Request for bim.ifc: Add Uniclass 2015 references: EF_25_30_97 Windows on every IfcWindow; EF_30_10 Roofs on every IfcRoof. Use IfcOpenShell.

First a look at what the model holds.

```python
import ifcopenshell

model = ifcopenshell.open("bim.ifc")
print(model.schema)
print("classifications:", [c.Name for c in model.by_type("IfcClassification")])
for ifc_class in ("IfcDoor", "IfcRoof", "IfcStair", "IfcWall", "IfcWindow"):
    print(ifc_class, len(model.by_type(ifc_class)))
```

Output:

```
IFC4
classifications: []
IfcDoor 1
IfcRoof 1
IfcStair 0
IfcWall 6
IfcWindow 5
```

```python
import ifcopenshell
import ifcopenshell.api.classification

model = ifcopenshell.open("bim.ifc")

system = ifcopenshell.api.classification.add_classification(model, classification="Uniclass 2015")

codes = {
    "IfcWindow": ("EF_25_30_97", "Windows"),
    "IfcRoof": ("EF_30_10", "Roofs"),
}
for ifc_class, (code, name) in codes.items():
    products = model.by_type(ifc_class)
    ifcopenshell.api.classification.add_reference(
        model, products=products, classification=system, identification=code, name=name
    )
    print(code, len(products))

model.write("bim_edited.ifc")
```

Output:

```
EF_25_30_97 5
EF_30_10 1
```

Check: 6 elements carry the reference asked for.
